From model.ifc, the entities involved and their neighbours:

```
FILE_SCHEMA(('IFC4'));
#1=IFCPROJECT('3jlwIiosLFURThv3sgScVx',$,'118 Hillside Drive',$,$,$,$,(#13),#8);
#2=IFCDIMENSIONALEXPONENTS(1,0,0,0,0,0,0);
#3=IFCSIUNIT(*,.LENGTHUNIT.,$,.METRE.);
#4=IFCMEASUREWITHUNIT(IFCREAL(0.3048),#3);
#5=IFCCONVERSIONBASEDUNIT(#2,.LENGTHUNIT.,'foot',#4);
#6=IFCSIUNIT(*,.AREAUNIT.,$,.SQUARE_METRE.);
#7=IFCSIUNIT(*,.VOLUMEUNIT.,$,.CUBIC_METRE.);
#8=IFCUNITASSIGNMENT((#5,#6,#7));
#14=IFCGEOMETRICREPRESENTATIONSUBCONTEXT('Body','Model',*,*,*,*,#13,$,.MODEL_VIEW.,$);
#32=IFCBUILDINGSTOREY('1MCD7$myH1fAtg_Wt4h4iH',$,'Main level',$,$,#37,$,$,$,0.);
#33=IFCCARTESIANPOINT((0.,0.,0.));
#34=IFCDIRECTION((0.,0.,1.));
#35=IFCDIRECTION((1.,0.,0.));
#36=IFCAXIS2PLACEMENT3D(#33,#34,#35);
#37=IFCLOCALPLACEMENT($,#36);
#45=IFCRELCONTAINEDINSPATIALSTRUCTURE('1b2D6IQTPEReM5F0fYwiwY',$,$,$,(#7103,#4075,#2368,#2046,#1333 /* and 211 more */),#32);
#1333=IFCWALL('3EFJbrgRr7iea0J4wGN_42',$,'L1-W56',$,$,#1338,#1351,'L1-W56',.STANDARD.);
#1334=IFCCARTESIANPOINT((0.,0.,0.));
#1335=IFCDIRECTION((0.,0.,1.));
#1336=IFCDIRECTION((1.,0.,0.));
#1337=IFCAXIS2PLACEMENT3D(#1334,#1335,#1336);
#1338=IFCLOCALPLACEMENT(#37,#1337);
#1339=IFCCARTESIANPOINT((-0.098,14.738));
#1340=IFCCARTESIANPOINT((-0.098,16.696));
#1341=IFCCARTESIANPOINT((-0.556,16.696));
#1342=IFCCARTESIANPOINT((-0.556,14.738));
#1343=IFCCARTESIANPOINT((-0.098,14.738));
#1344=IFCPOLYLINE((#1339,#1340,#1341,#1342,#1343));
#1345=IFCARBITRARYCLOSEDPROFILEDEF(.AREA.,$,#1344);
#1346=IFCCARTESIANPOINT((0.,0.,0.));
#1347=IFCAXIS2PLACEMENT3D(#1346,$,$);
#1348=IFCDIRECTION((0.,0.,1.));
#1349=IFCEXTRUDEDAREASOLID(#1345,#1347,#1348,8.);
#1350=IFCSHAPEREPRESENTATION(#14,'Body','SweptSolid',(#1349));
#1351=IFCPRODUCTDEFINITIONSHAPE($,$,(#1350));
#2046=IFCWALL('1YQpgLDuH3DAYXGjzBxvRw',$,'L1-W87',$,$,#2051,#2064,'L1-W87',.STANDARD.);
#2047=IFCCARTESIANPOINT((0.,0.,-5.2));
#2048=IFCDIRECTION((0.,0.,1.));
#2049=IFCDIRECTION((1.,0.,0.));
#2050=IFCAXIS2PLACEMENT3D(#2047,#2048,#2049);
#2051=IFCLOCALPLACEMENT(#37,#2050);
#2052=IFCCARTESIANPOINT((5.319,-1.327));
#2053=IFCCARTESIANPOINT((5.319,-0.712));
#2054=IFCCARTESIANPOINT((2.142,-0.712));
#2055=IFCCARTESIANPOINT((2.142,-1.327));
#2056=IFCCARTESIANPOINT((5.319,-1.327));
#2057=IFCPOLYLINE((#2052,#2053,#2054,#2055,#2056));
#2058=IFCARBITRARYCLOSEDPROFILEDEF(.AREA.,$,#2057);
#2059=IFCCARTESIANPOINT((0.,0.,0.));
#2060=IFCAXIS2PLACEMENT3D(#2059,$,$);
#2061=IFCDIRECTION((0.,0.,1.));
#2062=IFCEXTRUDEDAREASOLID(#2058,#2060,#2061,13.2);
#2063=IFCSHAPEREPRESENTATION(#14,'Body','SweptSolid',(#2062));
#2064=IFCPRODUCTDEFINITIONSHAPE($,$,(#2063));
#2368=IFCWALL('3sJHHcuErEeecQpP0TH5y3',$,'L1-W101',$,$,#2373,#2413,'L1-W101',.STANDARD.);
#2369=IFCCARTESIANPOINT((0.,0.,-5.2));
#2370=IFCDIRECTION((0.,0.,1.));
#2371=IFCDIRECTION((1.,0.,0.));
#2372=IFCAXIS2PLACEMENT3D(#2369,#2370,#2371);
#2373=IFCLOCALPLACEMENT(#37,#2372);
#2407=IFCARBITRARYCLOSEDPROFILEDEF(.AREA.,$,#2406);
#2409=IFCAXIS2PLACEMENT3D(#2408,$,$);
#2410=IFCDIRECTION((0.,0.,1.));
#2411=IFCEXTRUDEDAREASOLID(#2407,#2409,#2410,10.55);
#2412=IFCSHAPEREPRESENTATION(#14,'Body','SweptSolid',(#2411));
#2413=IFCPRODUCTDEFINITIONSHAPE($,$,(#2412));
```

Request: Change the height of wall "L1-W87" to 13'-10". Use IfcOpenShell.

```python
import ifcopenshell
import ifcopenshell.geom
import ifcopenshell.util.representation
import ifcopenshell.util.shape
import ifcopenshell.util.unit

model = ifcopenshell.open("model.ifc")
unit_scale = ifcopenshell.util.unit.calculate_unit_scale(model)
settings = ifcopenshell.geom.settings()


def volume(element):
    """Net volume in cubic metres, openings subtracted."""
    shape = ifcopenshell.geom.create_shape(settings, element)
    return ifcopenshell.util.shape.get_volume(shape.geometry)


wall = model.by_guid("1YQpgLDuH3DAYXGjzBxvRw")
before = volume(wall)

body = ifcopenshell.util.representation.get_representation(wall, "Model", "Body")
solid = body.Items[0]
old_height = solid.Depth
solid.Depth = 166 * 0.0254 / unit_scale
after = volume(wall)

print(f"height {old_height:g} -> {solid.Depth:g}, volume {before:.3f} -> {after:.3f} m3")

model.write("model-out.ifc")
```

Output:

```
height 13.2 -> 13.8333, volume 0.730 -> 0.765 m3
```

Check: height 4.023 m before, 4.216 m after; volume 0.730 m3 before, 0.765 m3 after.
